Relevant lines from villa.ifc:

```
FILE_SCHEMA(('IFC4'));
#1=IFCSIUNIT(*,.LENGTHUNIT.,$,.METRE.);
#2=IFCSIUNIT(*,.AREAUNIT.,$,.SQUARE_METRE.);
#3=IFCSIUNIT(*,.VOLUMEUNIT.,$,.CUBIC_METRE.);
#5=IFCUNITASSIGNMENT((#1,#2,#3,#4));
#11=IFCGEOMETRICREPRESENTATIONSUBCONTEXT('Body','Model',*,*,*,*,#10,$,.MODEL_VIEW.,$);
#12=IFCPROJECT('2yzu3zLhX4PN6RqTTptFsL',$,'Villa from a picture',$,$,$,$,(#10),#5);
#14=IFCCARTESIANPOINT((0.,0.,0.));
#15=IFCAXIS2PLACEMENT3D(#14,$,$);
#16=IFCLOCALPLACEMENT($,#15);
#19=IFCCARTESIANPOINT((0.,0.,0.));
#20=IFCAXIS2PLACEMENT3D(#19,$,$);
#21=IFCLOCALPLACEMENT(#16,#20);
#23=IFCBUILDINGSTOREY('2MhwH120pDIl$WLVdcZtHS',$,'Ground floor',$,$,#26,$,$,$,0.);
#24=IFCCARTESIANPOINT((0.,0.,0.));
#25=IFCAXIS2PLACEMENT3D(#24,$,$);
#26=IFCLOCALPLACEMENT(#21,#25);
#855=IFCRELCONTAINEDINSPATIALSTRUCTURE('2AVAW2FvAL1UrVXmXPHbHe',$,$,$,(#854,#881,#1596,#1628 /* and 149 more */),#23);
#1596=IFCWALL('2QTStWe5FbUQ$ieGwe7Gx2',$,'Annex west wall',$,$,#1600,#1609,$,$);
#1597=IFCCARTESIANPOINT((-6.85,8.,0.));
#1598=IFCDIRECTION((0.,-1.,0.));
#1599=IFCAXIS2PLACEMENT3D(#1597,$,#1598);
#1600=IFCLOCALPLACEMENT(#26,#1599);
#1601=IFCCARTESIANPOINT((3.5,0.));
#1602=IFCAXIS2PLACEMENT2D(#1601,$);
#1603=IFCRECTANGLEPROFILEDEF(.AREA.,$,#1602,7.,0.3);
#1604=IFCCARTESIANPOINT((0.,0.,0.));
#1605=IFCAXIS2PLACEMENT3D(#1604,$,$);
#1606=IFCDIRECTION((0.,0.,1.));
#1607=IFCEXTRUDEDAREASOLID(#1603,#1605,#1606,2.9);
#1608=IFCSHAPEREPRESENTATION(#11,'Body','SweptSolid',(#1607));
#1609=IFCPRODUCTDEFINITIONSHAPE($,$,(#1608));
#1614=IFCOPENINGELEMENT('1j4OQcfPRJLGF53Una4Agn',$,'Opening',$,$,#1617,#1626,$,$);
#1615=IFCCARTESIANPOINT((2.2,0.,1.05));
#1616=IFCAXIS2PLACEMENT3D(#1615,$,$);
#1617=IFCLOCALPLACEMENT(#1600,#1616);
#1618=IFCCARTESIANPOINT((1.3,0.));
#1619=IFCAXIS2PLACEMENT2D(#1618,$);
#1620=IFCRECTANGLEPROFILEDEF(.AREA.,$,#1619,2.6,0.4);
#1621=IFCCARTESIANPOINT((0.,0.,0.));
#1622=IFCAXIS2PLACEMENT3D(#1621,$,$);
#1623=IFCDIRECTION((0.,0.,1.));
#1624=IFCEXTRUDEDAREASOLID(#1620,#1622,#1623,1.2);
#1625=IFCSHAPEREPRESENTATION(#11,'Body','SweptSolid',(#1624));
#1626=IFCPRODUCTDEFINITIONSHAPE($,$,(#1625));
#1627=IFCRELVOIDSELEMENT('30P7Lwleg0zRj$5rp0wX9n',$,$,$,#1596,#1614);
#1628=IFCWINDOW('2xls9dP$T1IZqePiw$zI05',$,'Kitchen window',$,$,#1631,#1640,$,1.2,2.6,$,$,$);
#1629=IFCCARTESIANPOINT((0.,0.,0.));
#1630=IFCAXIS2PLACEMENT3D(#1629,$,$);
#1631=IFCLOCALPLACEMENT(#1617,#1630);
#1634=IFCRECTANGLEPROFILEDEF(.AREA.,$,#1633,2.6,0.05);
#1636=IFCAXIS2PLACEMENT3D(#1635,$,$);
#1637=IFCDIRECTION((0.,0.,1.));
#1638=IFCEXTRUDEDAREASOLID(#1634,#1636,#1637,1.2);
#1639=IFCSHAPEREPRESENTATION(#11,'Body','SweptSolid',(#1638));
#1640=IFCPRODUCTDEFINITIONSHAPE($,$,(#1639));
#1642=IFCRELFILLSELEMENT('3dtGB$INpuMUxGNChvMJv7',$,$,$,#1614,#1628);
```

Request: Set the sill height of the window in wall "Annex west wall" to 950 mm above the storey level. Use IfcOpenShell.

```python
import numpy as np
import ifcopenshell
import ifcopenshell.api.geometry
import ifcopenshell.geom
import ifcopenshell.util.element
import ifcopenshell.util.placement
import ifcopenshell.util.shape
import ifcopenshell.util.unit

model = ifcopenshell.open("villa.ifc")
unit_scale = ifcopenshell.util.unit.calculate_unit_scale(model)

window = model.by_guid("2xls9dP$T1IZqePiw$zI05")
opening = window.FillsVoids[0].RelatingOpeningElement
storey = ifcopenshell.util.element.get_container(window, ifc_class="IfcBuildingStorey")
level = ifcopenshell.util.placement.get_local_placement(storey.ObjectPlacement)[2, 3]

# The opening's origin need not be at the sill, so measure its lowest point.
shape = ifcopenshell.geom.create_shape(ifcopenshell.geom.settings(), opening)
bottom = ifcopenshell.util.shape.get_shape_bottom_elevation(shape, shape.geometry) / unit_scale
dz = level + 0.95 / unit_scale - bottom

shift = np.array([0.0, 0.0, dz])
# The window is placed relative to its opening, so it follows when the opening moves.
matrix = ifcopenshell.util.placement.get_local_placement(opening.ObjectPlacement)
matrix[:3, 3] += shift
ifcopenshell.api.geometry.edit_object_placement(
    model, product=opening, matrix=matrix, is_si=False, should_transform_children=True
)

print(f"moved by {dz * unit_scale:+.3f} m")

model.write("villa-out.ifc")
```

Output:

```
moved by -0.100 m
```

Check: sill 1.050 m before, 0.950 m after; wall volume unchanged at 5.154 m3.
